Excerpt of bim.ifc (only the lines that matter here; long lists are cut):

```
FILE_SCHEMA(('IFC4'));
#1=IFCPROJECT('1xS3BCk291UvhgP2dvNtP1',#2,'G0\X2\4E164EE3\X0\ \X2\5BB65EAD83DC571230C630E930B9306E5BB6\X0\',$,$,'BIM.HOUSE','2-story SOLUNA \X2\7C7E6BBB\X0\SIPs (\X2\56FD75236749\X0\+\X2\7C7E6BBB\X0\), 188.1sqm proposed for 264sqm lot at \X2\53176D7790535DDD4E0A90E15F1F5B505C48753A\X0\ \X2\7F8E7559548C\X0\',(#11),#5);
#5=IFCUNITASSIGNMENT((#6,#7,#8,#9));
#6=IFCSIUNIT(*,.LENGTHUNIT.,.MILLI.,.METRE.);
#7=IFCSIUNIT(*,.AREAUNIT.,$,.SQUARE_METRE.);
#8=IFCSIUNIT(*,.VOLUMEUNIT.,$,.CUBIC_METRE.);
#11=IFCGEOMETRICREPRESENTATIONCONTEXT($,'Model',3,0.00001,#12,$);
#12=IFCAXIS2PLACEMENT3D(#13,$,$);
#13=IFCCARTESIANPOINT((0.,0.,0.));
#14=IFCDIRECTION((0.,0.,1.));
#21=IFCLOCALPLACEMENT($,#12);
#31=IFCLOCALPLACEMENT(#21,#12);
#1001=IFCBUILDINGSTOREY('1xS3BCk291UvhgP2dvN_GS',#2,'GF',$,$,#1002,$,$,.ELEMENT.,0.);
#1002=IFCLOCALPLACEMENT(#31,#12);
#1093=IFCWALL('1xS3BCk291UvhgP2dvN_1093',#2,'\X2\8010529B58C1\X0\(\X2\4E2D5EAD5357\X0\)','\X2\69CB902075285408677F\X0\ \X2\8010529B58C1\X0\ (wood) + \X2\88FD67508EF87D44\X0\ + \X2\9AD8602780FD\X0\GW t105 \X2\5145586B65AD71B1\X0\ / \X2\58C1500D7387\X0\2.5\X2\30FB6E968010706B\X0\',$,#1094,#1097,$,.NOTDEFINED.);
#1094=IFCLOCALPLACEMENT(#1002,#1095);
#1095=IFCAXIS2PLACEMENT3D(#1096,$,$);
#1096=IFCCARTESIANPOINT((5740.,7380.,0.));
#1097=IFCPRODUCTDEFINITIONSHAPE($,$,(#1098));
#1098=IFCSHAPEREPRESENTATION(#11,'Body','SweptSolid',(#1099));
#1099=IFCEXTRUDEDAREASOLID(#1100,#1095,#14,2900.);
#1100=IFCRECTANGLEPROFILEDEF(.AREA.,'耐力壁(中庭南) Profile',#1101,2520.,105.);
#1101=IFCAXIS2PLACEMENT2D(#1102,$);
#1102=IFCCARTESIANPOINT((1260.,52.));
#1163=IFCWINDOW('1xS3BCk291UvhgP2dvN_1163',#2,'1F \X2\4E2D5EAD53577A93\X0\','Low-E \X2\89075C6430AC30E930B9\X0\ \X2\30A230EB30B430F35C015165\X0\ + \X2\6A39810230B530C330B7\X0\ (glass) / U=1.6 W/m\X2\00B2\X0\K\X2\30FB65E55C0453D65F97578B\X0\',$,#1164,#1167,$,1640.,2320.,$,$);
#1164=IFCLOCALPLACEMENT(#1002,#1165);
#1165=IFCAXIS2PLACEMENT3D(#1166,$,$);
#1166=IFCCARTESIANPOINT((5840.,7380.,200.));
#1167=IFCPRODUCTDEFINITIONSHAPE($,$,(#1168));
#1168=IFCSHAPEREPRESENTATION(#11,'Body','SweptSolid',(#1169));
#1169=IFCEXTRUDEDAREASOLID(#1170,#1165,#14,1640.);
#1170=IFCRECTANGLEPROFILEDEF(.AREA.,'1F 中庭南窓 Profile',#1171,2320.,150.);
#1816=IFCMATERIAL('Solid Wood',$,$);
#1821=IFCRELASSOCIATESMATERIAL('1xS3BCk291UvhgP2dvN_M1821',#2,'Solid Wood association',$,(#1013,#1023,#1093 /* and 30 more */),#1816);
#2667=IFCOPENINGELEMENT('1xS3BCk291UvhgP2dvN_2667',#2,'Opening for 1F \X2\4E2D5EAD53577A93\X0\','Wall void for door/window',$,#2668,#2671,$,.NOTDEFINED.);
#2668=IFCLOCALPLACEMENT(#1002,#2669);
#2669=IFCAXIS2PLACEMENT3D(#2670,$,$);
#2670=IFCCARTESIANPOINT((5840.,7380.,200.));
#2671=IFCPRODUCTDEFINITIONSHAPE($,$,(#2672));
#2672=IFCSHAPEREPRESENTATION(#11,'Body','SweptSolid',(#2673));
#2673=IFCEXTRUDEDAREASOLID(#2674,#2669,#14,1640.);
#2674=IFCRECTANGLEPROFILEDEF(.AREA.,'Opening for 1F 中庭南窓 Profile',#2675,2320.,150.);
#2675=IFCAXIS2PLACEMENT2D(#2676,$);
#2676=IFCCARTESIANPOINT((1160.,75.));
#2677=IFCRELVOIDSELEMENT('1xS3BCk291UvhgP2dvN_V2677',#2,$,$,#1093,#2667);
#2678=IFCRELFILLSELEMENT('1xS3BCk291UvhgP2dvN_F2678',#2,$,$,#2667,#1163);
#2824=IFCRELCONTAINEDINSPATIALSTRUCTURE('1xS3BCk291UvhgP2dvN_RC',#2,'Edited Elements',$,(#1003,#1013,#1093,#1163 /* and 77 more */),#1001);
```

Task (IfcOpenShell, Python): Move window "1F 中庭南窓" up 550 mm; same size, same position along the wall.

```python
import numpy as np
import ifcopenshell
import ifcopenshell.api.geometry
import ifcopenshell.util.placement
import ifcopenshell.util.unit

model = ifcopenshell.open("bim.ifc")
unit_scale = ifcopenshell.util.unit.calculate_unit_scale(model)

window = model.by_id(1163)
opening = window.FillsVoids[0].RelatingOpeningElement
dz = 0.55 / unit_scale

shift = np.array([0.0, 0.0, dz])
# The window is not placed relative to its opening, so move both.
for product in (opening, window):
    matrix = ifcopenshell.util.placement.get_local_placement(product.ObjectPlacement)
    matrix[:3, 3] += shift
    ifcopenshell.api.geometry.edit_object_placement(model, product=product, matrix=matrix, is_si=False)

print(f"moved by {dz * unit_scale:+.3f} m")

model.write("bim_rev.ifc")
```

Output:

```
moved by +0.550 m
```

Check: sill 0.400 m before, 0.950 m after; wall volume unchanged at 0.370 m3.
